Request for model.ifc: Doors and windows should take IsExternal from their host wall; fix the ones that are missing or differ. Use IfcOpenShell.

First a look at what the model holds.

```python
import ifcopenshell
import ifcopenshell.util.element

model = ifcopenshell.open("model.ifc")
print(model.schema)
seen = {}
for e in model.by_type("IfcDoor") + model.by_type("IfcWindow"):
    if not e.FillsVoids:
        continue
    host = e.FillsVoids[0].RelatingOpeningElement.VoidsElements[0].RelatingBuildingElement
    own = ifcopenshell.util.element.get_pset(e, f"Pset_{e.is_a()[3:].removesuffix('StandardCase')}Common", "IsExternal")
    wall = ifcopenshell.util.element.get_pset(host, "Pset_WallCommon", "IsExternal")
    seen[e.is_a(), own, wall] = seen.get((e.is_a(), own, wall), 0) + 1
for (cls, own, wall), count in sorted(seen.items(), key=str):
    print(count, cls, "IsExternal:", own, "| host wall:", wall)
```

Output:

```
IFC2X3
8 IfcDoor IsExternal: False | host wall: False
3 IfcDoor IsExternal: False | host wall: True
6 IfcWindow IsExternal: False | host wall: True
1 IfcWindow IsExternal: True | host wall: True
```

```python
import ifcopenshell
import ifcopenshell.api.pset
import ifcopenshell.util.element

model = ifcopenshell.open("model.ifc")

count = 0
for ifc_class, pset_name in (("IfcDoor", "Pset_DoorCommon"), ("IfcWindow", "Pset_WindowCommon")):
    for e in model.by_type(ifc_class):
        if not e.FillsVoids:
            continue
        host = e.FillsVoids[0].RelatingOpeningElement.VoidsElements[0].RelatingBuildingElement
        external = ifcopenshell.util.element.get_pset(host, "Pset_WallCommon", "IsExternal")
        if external is None or ifcopenshell.util.element.get_pset(e, pset_name, "IsExternal") == external:
            continue
        pset = ifcopenshell.api.pset.add_pset(model, product=e, name=pset_name)
        ifcopenshell.api.pset.edit_pset(model, pset=pset, properties={"IsExternal": external})
        count += 1

print(count, "updated")

model.write("model_updated.ifc")
```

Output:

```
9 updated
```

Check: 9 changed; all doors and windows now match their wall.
